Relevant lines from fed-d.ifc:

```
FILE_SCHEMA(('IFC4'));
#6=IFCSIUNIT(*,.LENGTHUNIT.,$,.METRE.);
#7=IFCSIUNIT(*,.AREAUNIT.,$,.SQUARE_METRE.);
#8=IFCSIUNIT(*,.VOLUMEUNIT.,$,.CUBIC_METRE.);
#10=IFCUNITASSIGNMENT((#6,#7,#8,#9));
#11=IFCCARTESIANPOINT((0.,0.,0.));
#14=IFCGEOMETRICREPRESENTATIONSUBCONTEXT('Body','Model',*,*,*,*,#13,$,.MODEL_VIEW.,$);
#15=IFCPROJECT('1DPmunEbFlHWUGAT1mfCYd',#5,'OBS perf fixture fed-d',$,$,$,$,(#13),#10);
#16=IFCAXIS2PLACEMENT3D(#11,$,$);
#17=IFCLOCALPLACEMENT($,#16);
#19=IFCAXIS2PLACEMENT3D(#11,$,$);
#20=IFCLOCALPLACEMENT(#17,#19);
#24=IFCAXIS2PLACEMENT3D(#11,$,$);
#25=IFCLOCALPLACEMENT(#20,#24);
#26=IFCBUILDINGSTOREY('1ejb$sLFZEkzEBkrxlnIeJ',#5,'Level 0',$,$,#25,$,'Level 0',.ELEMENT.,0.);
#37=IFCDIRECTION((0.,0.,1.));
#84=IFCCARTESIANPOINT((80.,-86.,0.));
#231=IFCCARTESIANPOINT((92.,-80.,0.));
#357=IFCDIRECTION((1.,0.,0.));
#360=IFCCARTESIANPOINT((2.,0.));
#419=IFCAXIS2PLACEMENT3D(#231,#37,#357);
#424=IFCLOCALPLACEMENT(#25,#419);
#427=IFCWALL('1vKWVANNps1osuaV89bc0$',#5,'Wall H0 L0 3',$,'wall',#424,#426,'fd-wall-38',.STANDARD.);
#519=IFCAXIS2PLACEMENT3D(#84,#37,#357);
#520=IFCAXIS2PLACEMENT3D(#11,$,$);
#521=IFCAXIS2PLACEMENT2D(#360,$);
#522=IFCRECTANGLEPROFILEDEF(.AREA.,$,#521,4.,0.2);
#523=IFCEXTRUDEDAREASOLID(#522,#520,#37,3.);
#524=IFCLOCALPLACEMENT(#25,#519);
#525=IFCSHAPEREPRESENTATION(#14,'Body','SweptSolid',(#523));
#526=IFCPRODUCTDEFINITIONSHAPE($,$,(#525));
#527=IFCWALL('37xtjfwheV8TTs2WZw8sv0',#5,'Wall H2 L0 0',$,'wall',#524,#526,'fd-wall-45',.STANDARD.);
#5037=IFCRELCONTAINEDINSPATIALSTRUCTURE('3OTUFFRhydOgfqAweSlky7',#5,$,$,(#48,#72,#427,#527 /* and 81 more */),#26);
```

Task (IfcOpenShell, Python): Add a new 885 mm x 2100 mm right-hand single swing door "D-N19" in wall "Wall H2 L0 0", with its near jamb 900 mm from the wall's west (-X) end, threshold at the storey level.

```python
import numpy as np
import ifcopenshell
import ifcopenshell.api.feature
import ifcopenshell.api.geometry
import ifcopenshell.api.root
import ifcopenshell.api.spatial
import ifcopenshell.geom
import ifcopenshell.util.element
import ifcopenshell.util.placement
import ifcopenshell.util.representation
import ifcopenshell.util.shape
import ifcopenshell.util.unit

model = ifcopenshell.open("fed-d.ifc")
unit_scale = ifcopenshell.util.unit.calculate_unit_scale(model)
settings = ifcopenshell.geom.settings()


def volume(element):
    """Net volume in cubic metres, openings subtracted."""
    shape = ifcopenshell.geom.create_shape(settings, element)
    return ifcopenshell.util.shape.get_volume(shape.geometry)


wall = model.by_guid("37xtjfwheV8TTs2WZw8sv0")
storey = ifcopenshell.util.element.get_container(wall, ifc_class="IfcBuildingStorey")
context = ifcopenshell.util.representation.get_context(model, "Model", "Body", "MODEL_VIEW")
before = volume(wall)

width, height, from_end, sill = 0.885, 2.1, 0.9, 0.0  # metres

# The wall runs along its own X axis, and the end named is its -X end.
wall_shape = ifcopenshell.geom.create_shape(settings, wall)
x, y, z = ifcopenshell.util.shape.get_vertices(wall_shape.geometry).T
start = x.min() + from_end
face, thickness = float(y.min()), float(y.max() - y.min())
wall_matrix = ifcopenshell.util.placement.get_local_placement(wall.ObjectPlacement)
level = ifcopenshell.util.placement.get_local_placement(storey.ObjectPlacement)[2, 3]


def in_wall(x, y):
    """Placement at x, y metres in the wall's axes, at sill height."""
    matrix = wall_matrix.copy()
    matrix[:, 3] = wall_matrix @ np.array([x / unit_scale, y / unit_scale, 0.0, 1.0])
    matrix[2, 3] = level + sill / unit_scale
    return matrix


# Opening: a box that overshoots both wall faces by 50 mm.
opening = ifcopenshell.api.root.create_entity(model, ifc_class="IfcOpeningElement", predefined_type="OPENING")
box = ifcopenshell.api.geometry.add_wall_representation(
    model, context=context, length=width, height=height, thickness=thickness + 0.1
)
ifcopenshell.api.geometry.assign_representation(model, product=opening, representation=box)
ifcopenshell.api.geometry.edit_object_placement(model, product=opening, matrix=in_wall(start, face - 0.05), is_si=False)
ifcopenshell.api.feature.add_feature(model, feature=opening, element=wall)

door = ifcopenshell.api.root.create_entity(model, ifc_class="IfcDoor", name="D-N19", predefined_type="DOOR")
door.OverallWidth, door.OverallHeight = width / unit_scale, height / unit_scale
door.OperationType = "SINGLE_SWING_RIGHT"
body = ifcopenshell.api.geometry.add_door_representation(
    model,
    context=context,
    overall_width=door.OverallWidth,
    overall_height=door.OverallHeight,
    operation_type="SINGLE_SWING_RIGHT",
    lining_properties={"LiningDepth": thickness / unit_scale, "ThresholdDepth": thickness / unit_scale},
)
ifcopenshell.api.geometry.assign_representation(model, product=door, representation=body)
ifcopenshell.api.spatial.assign_container(model, products=[door], relating_structure=storey)
ifcopenshell.api.feature.add_filling(model, opening=opening, element=door)

# The lining spans the wall, so the door starts at the wall face.
ifcopenshell.api.geometry.edit_object_placement(model, product=door, matrix=in_wall(start, face), is_si=False)

after = volume(wall)

print(f"wall volume {before:.3f} -> {after:.3f} m3")

model.write("fed-d_v2.ifc")
```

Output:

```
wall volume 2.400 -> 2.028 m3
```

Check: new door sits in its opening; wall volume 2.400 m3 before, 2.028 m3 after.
